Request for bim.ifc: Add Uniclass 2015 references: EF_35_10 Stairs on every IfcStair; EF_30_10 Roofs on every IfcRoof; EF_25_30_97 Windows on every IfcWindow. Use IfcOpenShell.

First a look at what the model holds.

```python
import ifcopenshell

model = ifcopenshell.open("bim.ifc")
print(model.schema)
print("classifications:", [c.Name for c in model.by_type("IfcClassification")])
for ifc_class in ("IfcDoor", "IfcRoof", "IfcStair", "IfcWall", "IfcWindow"):
    print(ifc_class, len(model.by_type(ifc_class)))
```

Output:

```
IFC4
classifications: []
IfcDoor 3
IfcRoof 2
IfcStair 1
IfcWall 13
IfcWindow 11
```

```python
import ifcopenshell
import ifcopenshell.api.classification

model = ifcopenshell.open("bim.ifc")

system = ifcopenshell.api.classification.add_classification(model, classification="Uniclass 2015")

codes = {
    "IfcStair": ("EF_35_10", "Stairs"),
    "IfcRoof": ("EF_30_10", "Roofs"),
    "IfcWindow": ("EF_25_30_97", "Windows"),
}
for ifc_class, (code, name) in codes.items():
    products = model.by_type(ifc_class)
    ifcopenshell.api.classification.add_reference(
        model, products=products, classification=system, identification=code, name=name
    )
    print(code, len(products))

model.write("bim_updated.ifc")
```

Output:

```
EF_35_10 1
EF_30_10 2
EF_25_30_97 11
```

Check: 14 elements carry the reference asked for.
